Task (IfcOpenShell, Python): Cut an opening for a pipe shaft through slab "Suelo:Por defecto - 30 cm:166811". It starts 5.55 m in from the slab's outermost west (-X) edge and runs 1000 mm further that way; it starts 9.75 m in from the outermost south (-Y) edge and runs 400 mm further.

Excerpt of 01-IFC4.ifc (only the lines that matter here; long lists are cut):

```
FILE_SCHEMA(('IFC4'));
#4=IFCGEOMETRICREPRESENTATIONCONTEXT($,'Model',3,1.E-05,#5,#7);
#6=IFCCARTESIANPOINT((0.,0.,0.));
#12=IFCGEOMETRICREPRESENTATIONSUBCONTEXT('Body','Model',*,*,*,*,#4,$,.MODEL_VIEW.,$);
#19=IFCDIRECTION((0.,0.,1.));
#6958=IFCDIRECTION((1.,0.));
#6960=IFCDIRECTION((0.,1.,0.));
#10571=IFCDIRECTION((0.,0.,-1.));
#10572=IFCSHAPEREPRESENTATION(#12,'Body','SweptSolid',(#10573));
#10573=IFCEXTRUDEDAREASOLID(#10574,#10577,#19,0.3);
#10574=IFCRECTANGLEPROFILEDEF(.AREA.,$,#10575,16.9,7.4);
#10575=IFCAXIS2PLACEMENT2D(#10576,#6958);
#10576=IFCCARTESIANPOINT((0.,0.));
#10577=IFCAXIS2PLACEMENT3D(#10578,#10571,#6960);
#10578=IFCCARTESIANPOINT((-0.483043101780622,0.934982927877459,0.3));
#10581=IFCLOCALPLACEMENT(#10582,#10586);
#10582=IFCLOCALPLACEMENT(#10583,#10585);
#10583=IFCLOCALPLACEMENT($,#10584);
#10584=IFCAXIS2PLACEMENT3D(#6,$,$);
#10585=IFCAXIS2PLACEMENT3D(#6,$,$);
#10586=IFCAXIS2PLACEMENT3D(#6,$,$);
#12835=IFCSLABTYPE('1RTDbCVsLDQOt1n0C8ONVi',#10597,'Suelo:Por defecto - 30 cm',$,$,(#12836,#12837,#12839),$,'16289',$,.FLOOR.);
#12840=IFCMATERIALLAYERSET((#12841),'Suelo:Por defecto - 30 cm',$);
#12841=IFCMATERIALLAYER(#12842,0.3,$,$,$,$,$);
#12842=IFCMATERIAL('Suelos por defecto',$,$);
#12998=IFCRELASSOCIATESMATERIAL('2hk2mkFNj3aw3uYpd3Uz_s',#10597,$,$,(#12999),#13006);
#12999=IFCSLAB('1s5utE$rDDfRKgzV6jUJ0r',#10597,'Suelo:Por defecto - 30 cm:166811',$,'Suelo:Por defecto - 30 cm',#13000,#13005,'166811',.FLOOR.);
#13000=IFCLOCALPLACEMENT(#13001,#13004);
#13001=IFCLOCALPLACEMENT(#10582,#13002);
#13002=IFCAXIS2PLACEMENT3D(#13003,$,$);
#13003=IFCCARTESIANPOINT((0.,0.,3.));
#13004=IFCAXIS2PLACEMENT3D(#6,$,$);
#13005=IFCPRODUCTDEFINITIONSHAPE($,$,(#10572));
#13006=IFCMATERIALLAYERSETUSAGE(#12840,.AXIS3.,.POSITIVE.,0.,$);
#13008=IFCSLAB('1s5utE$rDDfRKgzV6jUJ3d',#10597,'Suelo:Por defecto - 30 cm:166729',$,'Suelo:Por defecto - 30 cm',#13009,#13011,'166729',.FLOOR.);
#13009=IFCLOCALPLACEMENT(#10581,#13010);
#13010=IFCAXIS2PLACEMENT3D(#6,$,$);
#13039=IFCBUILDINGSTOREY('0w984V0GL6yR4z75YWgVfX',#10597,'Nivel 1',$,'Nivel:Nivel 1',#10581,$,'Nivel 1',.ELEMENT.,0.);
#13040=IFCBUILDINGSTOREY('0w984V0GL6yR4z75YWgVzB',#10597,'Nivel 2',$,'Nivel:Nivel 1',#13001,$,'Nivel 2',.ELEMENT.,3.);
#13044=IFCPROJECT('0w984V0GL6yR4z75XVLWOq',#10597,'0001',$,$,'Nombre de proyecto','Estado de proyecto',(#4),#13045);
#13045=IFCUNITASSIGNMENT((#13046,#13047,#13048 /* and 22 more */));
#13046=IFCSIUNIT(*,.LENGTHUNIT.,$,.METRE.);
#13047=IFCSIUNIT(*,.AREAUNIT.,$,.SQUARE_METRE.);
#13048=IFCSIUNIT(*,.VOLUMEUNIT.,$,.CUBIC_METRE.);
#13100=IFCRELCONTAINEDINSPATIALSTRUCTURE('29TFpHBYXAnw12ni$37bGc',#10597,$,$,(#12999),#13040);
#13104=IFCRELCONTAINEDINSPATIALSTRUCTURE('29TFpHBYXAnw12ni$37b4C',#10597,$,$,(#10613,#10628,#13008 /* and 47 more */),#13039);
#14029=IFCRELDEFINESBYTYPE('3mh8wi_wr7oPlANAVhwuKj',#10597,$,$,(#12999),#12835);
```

```python
import numpy as np
import ifcopenshell
import ifcopenshell.api.feature
import ifcopenshell.api.geometry
import ifcopenshell.api.root
import ifcopenshell.geom
import ifcopenshell.util.placement
import ifcopenshell.util.representation
import ifcopenshell.util.shape
import ifcopenshell.util.unit

model = ifcopenshell.open("01-IFC4.ifc")
unit_scale = ifcopenshell.util.unit.calculate_unit_scale(model)
settings = ifcopenshell.geom.settings()


def volume(element):
    """Net volume in cubic metres, openings subtracted."""
    shape = ifcopenshell.geom.create_shape(settings, element)
    return ifcopenshell.util.shape.get_volume(shape.geometry)


slab = model.by_guid("1s5utE$rDDfRKgzV6jUJ0r")
before = volume(slab)

# Extent in the slab's own axes, in metres. The edges named are its -X and -Y sides.
slab_shape = ifcopenshell.geom.create_shape(settings, slab)
vertices = ifcopenshell.util.shape.get_vertices(slab_shape.geometry)
x_min, y_min, bottom = vertices.min(axis=0)
top = vertices[:, 2].max()

opening = ifcopenshell.api.root.create_entity(model, ifc_class="IfcOpeningElement", name="Pipe shaft opening", predefined_type="OPENING")
context = ifcopenshell.util.representation.get_context(model, "Model", "Body", "MODEL_VIEW")
width, depth = 1, 0.4
outline = [(0.0, 0.0), (width, 0.0), (width, depth), (0.0, depth), (0.0, 0.0)]
# Overshoot both faces by 50 mm so the cut is clean.
shape = ifcopenshell.api.geometry.add_slab_representation(
    model, context=context, depth=top - bottom + 0.1, polyline=outline
)
ifcopenshell.api.geometry.assign_representation(model, product=opening, representation=shape)

matrix = ifcopenshell.util.placement.get_local_placement(slab.ObjectPlacement)
matrix[:, 3] = matrix @ np.append(np.array([x_min + 5.55, y_min + 9.75, bottom - 0.05]) / unit_scale, 1.0)
ifcopenshell.api.geometry.edit_object_placement(model, product=opening, matrix=matrix, is_si=False)
ifcopenshell.api.feature.add_feature(model, feature=opening, element=slab)

after = volume(slab)

print(f"slab volume {before:.3f} -> {after:.3f} m3")

model.write("01-IFC4_updated.ifc")
```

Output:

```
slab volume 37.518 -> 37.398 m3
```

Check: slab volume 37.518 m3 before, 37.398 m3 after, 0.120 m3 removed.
